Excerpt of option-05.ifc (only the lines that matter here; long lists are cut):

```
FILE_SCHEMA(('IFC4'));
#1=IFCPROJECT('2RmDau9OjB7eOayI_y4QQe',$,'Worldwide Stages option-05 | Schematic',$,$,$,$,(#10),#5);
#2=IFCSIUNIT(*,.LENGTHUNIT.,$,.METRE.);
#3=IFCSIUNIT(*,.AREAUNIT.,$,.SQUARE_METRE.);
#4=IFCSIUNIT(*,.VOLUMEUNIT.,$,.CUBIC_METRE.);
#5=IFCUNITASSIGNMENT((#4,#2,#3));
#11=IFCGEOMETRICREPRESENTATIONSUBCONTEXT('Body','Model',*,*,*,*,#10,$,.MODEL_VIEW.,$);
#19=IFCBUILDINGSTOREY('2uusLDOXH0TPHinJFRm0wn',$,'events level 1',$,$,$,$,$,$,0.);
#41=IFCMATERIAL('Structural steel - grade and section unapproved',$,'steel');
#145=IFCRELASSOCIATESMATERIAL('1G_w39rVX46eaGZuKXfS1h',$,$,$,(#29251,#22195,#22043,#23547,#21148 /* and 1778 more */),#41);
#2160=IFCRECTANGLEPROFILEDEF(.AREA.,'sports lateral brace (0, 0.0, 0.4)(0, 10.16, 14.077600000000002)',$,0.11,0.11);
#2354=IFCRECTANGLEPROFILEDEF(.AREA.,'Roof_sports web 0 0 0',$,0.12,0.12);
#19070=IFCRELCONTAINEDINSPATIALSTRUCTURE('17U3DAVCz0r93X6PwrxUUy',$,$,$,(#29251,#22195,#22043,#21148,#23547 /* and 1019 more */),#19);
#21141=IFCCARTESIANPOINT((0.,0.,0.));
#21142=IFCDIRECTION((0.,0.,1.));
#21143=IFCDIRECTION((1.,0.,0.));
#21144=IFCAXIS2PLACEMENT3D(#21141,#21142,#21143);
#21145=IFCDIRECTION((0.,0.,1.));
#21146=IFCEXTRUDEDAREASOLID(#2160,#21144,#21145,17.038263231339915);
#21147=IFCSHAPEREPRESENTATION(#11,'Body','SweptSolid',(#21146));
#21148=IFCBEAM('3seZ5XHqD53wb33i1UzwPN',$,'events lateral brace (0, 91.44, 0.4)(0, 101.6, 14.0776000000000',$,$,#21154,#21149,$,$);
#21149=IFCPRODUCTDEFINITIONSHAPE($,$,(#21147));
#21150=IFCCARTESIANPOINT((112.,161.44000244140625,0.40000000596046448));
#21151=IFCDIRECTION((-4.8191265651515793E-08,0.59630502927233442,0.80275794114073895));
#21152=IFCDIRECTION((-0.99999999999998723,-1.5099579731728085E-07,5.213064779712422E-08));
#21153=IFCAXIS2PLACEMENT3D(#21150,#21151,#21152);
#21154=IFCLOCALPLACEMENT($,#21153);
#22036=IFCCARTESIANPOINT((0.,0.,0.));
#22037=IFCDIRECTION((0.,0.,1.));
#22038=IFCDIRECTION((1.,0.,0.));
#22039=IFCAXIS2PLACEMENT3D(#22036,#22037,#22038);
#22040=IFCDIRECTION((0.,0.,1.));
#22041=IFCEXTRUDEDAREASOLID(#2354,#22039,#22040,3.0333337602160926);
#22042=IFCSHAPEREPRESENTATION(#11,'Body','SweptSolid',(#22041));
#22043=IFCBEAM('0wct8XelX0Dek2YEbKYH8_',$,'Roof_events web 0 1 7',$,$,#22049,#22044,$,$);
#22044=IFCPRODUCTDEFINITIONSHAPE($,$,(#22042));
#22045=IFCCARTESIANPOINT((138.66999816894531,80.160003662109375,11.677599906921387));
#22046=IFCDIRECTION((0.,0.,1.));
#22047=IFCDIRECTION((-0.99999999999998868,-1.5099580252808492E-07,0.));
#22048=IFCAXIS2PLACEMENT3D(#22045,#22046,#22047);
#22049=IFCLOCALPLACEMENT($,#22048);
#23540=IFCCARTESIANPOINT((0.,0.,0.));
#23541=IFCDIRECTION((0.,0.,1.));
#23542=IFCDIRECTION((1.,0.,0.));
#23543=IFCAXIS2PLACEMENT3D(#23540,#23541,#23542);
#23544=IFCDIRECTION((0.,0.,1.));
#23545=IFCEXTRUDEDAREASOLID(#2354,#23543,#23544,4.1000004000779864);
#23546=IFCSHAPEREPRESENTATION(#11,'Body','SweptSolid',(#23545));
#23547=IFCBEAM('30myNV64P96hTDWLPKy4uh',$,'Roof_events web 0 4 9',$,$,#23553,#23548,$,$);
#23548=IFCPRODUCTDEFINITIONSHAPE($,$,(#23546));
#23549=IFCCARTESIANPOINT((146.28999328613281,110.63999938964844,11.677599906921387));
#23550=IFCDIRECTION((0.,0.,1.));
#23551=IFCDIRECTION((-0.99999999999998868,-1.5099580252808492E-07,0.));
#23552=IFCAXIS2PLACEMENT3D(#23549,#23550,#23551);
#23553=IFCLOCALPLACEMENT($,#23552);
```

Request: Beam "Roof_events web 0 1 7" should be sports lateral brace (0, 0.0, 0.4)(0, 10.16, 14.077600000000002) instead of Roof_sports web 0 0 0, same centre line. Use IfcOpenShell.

```python
import ifcopenshell
import ifcopenshell.util.element
import ifcopenshell.util.representation

model = ifcopenshell.open("option-05.ifc")

member = model.by_id(22043)
source = next(p for p in model.by_type("IfcRectangleProfileDef") if p.ProfileName == "sports lateral brace (0, 0.0, 0.4)(0, 10.16, 14.077600000000002)")

body = ifcopenshell.util.representation.get_representation(member, "Model", "Body")
solid = body.Items[0]
old_profile = solid.SweptArea

# Copy the section's sizes but keep this member's own profile position.
profile = ifcopenshell.util.element.copy(model, source)
profile.Position = old_profile.Position
solid.SweptArea = profile
if not model.get_total_inverses(old_profile):
    ifcopenshell.util.element.remove_deep2(model, old_profile)

print(solid.SweptArea)

model.write("option-05_rev.ifc")
```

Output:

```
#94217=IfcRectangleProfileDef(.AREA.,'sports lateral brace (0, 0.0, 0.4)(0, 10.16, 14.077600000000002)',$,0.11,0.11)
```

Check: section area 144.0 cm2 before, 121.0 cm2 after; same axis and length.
